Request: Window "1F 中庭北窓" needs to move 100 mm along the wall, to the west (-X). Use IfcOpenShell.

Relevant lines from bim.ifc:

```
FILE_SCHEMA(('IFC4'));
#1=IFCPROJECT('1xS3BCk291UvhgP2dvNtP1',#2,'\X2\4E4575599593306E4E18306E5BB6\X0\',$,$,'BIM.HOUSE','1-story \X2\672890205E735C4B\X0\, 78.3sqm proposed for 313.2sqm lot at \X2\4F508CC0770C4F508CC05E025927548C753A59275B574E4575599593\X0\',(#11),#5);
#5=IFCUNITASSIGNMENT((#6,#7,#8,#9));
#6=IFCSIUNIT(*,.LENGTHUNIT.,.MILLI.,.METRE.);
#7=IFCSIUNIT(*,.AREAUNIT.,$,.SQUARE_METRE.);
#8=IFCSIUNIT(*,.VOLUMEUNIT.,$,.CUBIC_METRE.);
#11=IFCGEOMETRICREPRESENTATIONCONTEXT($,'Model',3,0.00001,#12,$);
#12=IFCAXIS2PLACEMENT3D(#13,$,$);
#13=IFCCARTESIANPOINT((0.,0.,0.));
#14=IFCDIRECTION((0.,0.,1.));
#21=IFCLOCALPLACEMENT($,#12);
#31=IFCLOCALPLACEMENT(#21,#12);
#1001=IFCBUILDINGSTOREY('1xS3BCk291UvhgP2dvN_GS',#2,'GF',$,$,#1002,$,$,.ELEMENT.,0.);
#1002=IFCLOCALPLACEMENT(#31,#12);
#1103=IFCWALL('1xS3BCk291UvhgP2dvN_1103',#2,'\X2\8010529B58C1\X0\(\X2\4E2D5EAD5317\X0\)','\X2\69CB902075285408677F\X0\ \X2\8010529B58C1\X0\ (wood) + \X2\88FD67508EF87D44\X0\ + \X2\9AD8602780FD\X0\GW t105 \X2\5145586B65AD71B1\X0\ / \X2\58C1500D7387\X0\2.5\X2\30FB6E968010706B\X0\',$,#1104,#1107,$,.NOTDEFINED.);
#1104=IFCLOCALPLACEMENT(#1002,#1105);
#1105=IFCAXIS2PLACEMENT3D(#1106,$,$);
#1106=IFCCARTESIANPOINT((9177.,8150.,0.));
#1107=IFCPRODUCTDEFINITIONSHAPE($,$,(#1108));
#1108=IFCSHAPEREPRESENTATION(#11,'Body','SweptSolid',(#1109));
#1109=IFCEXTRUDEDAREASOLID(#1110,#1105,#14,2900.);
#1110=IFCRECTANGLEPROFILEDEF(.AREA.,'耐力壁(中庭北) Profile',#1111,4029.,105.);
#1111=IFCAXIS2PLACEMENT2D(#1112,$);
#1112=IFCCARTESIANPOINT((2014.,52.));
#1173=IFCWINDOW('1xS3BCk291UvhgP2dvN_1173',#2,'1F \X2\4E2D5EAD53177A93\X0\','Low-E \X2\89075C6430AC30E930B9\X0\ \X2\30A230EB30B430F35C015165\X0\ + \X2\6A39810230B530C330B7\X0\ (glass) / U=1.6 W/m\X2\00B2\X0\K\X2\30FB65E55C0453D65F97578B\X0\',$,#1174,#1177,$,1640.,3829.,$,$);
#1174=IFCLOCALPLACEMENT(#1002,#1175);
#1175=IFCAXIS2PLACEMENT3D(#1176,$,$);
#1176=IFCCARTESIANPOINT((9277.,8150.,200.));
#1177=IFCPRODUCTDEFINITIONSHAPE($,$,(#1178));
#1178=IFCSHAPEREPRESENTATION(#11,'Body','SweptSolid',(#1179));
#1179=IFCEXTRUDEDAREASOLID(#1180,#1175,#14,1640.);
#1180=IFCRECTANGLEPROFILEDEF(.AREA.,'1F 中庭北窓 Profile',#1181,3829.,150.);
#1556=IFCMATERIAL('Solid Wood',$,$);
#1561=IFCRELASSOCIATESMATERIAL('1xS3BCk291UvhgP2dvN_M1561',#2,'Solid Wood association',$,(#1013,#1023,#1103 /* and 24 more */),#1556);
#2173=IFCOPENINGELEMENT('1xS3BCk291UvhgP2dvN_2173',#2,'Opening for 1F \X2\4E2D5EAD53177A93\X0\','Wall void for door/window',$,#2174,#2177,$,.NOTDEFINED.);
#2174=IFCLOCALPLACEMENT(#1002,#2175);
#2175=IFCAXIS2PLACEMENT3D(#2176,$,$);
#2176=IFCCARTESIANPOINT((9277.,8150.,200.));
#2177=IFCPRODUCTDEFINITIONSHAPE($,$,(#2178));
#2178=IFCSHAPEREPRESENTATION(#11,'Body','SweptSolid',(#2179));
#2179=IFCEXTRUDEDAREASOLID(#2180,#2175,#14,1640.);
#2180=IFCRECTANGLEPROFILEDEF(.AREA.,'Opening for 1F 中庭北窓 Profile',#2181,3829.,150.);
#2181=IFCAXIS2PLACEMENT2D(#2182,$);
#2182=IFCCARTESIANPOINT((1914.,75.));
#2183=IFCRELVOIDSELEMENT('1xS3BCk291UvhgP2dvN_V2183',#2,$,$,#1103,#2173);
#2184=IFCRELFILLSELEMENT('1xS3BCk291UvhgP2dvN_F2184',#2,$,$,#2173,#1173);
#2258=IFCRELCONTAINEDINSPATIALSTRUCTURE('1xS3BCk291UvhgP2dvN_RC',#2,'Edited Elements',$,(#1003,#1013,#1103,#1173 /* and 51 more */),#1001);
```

```python
import ifcopenshell
import ifcopenshell.api.geometry
import ifcopenshell.util.placement

model = ifcopenshell.open("bim.ifc")

window = model.by_guid("1xS3BCk291UvhgP2dvN_1173")
opening = window.FillsVoids[0].RelatingOpeningElement
wall = opening.VoidsElements[0].RelatingBuildingElement

wall_matrix = ifcopenshell.util.placement.get_local_placement(wall.ObjectPlacement)
shift = wall_matrix[:3, 0] * -100.0
before = ifcopenshell.util.placement.get_local_placement(window.ObjectPlacement)[:3, 3].copy()

# The window is not placed relative to its opening, so move both.
for product in (opening, window):
    matrix = ifcopenshell.util.placement.get_local_placement(product.ObjectPlacement)
    matrix[:3, 3] += shift
    ifcopenshell.api.geometry.edit_object_placement(model, product=product, matrix=matrix, is_si=False)

after = ifcopenshell.util.placement.get_local_placement(window.ObjectPlacement)[:3, 3]
print("window moved by", (after - before).round(3) + 0.0)

model.write("bim_v2.ifc")
```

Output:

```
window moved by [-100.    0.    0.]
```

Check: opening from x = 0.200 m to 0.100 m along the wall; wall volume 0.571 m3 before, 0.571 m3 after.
